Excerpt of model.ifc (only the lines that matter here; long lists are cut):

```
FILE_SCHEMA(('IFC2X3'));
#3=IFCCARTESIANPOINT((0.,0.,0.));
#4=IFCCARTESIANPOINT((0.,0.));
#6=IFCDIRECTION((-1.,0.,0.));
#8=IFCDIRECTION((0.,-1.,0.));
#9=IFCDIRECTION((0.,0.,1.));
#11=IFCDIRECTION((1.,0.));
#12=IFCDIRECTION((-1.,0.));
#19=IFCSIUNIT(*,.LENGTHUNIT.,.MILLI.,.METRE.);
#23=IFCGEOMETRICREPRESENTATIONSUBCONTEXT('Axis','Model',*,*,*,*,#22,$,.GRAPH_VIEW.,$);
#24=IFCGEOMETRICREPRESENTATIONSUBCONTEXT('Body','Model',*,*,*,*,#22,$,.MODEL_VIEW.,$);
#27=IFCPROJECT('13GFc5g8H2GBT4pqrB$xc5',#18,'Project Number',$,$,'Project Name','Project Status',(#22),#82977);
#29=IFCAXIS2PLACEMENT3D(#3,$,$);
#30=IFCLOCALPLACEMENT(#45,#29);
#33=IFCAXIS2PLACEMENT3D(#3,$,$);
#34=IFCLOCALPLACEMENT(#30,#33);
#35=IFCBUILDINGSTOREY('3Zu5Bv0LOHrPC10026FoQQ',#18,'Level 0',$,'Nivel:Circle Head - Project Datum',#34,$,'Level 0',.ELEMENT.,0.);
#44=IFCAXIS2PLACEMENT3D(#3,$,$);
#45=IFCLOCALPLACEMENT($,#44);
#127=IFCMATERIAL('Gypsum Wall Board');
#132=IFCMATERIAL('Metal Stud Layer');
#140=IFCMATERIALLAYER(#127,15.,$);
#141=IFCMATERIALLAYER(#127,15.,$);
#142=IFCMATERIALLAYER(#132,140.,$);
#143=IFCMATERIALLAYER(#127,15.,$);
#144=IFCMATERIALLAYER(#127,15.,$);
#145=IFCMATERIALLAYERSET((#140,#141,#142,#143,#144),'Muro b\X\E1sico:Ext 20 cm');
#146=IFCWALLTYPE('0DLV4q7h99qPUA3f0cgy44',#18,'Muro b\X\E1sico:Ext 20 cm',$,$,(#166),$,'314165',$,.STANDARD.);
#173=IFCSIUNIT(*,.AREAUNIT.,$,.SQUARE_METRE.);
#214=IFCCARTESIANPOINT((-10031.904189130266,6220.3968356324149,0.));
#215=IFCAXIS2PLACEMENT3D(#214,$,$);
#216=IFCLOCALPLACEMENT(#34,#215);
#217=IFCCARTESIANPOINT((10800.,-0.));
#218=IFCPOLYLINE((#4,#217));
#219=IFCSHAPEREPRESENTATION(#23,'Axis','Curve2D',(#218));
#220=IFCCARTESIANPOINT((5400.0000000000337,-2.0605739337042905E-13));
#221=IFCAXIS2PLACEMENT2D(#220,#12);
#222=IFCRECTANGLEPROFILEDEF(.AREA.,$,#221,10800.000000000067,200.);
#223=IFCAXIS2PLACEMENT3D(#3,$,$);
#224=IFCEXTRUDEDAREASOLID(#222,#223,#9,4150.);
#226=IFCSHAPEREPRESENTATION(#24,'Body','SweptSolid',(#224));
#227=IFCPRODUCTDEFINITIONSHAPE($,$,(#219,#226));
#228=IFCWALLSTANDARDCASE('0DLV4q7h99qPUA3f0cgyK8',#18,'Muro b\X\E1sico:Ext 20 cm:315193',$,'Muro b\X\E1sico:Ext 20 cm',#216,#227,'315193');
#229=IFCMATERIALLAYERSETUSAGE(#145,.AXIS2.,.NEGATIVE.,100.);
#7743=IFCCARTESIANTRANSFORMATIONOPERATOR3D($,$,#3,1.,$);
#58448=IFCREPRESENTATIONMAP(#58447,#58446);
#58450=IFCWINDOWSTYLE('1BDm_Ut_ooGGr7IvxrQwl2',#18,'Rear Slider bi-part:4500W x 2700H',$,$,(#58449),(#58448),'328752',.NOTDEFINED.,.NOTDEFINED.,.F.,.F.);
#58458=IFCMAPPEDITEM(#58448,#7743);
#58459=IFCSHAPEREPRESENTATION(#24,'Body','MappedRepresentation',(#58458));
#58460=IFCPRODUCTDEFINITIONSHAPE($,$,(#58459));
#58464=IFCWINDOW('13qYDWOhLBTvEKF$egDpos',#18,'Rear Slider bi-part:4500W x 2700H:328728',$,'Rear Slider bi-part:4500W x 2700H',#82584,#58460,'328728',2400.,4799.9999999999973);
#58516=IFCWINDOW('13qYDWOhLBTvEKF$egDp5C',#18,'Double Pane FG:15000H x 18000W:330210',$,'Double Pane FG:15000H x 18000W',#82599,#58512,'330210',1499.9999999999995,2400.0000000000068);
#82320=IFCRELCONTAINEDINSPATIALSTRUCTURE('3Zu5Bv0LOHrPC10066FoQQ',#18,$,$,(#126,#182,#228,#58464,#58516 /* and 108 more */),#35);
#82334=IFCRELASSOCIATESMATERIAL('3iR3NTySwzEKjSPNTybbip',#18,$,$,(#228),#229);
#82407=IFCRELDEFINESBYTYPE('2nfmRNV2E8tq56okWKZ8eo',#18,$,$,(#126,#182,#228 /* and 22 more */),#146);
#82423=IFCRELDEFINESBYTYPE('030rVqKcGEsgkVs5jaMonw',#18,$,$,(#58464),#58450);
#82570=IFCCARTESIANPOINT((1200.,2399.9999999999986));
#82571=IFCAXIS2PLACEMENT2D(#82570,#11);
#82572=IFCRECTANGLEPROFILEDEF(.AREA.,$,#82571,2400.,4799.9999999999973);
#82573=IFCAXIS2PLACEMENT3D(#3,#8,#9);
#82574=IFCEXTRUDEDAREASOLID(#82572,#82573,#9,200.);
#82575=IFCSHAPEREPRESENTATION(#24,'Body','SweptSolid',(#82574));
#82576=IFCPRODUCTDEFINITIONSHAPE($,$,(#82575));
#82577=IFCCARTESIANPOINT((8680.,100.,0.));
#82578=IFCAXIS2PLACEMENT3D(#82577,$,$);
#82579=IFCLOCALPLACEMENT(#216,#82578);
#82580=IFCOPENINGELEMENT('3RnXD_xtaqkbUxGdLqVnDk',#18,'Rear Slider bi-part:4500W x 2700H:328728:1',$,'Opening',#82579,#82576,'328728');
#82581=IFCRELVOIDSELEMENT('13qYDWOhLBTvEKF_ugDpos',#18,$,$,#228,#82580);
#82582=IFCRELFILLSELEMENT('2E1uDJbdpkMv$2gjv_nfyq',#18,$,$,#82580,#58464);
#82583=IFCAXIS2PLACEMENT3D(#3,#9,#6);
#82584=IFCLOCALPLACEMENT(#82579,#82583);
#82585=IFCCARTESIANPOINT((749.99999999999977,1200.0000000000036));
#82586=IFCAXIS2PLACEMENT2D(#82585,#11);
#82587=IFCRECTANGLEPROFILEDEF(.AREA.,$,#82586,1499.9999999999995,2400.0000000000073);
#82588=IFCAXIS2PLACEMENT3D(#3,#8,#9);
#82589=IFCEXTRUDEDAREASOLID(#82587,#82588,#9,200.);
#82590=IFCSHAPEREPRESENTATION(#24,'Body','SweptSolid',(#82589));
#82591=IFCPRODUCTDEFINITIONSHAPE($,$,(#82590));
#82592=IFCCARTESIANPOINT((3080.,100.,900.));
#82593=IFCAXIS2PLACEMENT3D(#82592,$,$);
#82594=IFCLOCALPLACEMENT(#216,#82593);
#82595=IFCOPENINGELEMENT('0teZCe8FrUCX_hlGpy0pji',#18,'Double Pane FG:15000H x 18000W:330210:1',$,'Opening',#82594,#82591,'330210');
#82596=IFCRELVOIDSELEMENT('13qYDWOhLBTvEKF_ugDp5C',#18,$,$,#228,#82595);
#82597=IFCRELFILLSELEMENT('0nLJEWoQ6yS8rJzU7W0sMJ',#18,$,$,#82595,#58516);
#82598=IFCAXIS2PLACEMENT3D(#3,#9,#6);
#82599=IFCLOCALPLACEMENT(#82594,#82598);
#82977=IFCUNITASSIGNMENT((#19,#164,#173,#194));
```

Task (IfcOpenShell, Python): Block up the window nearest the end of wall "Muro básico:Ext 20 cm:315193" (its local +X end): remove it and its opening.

```python
import ifcopenshell
import ifcopenshell.api.feature
import ifcopenshell.api.root
import ifcopenshell.geom
import ifcopenshell.util.shape

model = ifcopenshell.open("model.ifc")
settings = ifcopenshell.geom.settings()


def volume(element):
    """Net volume in cubic metres, openings subtracted."""
    shape = ifcopenshell.geom.create_shape(settings, element)
    return ifcopenshell.util.shape.get_volume(shape.geometry)


window = model.by_guid("13qYDWOhLBTvEKF$egDpos")
opening = window.FillsVoids[0].RelatingOpeningElement
wall = opening.VoidsElements[0].RelatingBuildingElement
before = volume(wall)

ifcopenshell.api.root.remove_product(model, product=window)
ifcopenshell.api.feature.remove_feature(model, feature=opening)

after = volume(wall)

print(f"wall volume {before:.3f} -> {after:.3f} m3")

model.write("model_v2.ifc")
```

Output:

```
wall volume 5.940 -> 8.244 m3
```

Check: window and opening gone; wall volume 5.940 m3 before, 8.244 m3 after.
